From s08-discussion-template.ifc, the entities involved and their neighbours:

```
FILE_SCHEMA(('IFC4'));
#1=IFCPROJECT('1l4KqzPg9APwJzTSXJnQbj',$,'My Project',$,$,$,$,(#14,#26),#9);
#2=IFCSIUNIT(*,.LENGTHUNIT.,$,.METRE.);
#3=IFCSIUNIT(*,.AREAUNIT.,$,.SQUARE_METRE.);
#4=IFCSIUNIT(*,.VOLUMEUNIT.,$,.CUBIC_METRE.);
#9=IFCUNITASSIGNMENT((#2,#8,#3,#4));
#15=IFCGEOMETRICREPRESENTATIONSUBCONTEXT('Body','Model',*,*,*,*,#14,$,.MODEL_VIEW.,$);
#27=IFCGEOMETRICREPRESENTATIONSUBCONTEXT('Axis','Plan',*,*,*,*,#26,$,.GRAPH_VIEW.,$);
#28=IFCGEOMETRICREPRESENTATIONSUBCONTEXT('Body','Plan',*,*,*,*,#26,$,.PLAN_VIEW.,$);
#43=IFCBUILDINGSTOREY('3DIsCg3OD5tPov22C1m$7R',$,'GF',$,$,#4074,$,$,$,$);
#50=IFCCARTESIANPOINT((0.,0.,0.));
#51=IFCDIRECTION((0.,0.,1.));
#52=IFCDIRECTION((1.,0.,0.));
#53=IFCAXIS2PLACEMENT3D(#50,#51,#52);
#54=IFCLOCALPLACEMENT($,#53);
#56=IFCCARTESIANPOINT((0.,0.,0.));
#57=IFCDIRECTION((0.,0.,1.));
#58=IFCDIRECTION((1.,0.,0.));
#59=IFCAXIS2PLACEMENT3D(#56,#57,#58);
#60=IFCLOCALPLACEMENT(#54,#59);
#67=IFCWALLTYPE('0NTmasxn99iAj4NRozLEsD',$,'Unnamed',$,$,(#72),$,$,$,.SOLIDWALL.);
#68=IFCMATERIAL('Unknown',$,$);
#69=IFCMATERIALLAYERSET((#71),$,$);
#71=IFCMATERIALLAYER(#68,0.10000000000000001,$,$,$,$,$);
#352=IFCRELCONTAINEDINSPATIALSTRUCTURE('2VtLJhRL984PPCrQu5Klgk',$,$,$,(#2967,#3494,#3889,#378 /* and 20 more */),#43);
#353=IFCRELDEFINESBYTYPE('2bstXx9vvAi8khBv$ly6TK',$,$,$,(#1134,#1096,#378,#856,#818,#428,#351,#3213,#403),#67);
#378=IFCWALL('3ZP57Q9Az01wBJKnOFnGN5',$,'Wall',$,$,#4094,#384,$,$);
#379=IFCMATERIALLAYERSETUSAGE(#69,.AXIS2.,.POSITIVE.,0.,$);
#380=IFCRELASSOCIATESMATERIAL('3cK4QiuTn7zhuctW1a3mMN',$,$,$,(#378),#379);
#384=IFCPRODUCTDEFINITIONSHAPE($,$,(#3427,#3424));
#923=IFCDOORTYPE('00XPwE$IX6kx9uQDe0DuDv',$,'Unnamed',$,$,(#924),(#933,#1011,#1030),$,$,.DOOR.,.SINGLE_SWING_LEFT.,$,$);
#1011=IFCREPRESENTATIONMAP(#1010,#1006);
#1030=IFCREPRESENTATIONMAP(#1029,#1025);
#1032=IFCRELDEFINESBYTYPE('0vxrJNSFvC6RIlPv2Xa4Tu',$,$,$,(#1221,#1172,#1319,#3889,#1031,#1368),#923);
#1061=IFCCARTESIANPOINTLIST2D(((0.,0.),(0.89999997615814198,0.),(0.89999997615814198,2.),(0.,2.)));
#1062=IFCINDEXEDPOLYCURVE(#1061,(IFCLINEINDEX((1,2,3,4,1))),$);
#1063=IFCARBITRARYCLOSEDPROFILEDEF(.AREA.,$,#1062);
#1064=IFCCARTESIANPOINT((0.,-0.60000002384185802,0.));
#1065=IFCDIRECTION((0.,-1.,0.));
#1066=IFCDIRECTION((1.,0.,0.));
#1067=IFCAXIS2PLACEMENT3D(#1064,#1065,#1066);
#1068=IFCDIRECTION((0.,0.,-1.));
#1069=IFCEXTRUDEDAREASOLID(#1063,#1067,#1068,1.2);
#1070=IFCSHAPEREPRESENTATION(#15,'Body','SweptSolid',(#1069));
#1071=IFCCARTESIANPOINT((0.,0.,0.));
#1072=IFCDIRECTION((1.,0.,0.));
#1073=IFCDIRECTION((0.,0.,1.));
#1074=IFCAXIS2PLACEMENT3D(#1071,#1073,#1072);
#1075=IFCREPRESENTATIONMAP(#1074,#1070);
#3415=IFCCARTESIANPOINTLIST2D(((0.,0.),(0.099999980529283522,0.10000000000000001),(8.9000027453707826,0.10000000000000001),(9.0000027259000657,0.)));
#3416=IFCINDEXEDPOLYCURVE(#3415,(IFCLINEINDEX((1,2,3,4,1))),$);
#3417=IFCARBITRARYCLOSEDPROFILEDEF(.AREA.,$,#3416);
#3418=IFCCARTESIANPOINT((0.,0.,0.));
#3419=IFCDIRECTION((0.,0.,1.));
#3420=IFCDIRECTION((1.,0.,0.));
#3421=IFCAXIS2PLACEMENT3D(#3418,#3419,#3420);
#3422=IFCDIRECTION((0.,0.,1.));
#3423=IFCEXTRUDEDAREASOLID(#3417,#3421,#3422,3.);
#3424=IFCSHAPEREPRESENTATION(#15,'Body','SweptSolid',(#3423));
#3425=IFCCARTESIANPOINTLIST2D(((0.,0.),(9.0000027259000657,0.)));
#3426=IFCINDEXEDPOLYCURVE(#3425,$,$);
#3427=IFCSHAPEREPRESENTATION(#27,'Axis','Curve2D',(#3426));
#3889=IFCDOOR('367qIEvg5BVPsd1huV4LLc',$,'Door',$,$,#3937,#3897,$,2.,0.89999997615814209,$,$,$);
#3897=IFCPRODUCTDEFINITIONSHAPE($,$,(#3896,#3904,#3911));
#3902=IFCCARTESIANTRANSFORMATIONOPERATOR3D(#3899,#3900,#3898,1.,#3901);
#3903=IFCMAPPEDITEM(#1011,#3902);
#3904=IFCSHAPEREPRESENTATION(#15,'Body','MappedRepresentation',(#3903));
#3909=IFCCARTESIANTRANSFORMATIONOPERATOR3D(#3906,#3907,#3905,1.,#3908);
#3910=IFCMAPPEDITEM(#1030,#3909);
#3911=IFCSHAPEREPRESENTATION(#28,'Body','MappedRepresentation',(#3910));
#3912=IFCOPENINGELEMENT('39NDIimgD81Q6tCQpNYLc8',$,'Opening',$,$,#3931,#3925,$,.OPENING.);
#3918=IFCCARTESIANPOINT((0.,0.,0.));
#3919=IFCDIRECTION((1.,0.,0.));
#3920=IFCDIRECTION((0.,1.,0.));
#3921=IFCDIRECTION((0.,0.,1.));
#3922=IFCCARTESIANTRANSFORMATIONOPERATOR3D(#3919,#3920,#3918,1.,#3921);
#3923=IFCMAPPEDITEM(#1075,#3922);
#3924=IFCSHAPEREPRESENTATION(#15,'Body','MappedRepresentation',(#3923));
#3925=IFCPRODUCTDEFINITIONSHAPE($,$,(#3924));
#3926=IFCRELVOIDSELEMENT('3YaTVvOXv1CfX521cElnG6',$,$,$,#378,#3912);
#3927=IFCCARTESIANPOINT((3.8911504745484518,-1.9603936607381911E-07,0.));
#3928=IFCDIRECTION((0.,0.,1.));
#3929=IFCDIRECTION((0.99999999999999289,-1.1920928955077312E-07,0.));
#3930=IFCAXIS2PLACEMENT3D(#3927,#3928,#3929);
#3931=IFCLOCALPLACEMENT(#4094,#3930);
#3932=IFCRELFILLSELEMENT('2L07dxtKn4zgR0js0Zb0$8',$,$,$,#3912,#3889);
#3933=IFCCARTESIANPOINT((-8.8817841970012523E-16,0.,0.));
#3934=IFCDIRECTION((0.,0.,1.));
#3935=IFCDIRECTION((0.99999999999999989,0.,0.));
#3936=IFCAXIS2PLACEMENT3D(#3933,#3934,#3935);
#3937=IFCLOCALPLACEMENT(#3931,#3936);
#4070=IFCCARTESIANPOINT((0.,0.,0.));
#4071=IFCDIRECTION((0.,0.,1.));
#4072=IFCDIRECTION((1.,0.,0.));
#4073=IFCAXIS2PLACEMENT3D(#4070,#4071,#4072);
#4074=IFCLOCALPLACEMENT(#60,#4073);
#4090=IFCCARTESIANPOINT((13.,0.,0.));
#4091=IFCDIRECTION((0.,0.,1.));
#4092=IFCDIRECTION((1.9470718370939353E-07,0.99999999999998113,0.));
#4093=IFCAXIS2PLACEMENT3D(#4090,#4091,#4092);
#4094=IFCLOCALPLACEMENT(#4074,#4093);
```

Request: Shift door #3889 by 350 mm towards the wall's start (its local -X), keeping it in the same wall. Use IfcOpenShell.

```python
import ifcopenshell
import ifcopenshell.api.geometry
import ifcopenshell.util.placement
import ifcopenshell.util.unit

model = ifcopenshell.open("s08-discussion-template.ifc")
unit_scale = ifcopenshell.util.unit.calculate_unit_scale(model)

door = model.by_id(3889)
opening = door.FillsVoids[0].RelatingOpeningElement
wall = opening.VoidsElements[0].RelatingBuildingElement

wall_matrix = ifcopenshell.util.placement.get_local_placement(wall.ObjectPlacement)
shift = wall_matrix[:3, 0] * -0.35 / unit_scale
before = ifcopenshell.util.placement.get_local_placement(door.ObjectPlacement)[:3, 3].copy()

# The door is placed relative to its opening, so it follows when the opening moves.
matrix = ifcopenshell.util.placement.get_local_placement(opening.ObjectPlacement)
matrix[:3, 3] += shift
ifcopenshell.api.geometry.edit_object_placement(
    model, product=opening, matrix=matrix, is_si=False, should_transform_children=True
)

after = ifcopenshell.util.placement.get_local_placement(door.ObjectPlacement)[:3, 3]
print("door moved by", (after - before).round(3) + 0.0)

model.write("s08-discussion-template_rev.ifc")
```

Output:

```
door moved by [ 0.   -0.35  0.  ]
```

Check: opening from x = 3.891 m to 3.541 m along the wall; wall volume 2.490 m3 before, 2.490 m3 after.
